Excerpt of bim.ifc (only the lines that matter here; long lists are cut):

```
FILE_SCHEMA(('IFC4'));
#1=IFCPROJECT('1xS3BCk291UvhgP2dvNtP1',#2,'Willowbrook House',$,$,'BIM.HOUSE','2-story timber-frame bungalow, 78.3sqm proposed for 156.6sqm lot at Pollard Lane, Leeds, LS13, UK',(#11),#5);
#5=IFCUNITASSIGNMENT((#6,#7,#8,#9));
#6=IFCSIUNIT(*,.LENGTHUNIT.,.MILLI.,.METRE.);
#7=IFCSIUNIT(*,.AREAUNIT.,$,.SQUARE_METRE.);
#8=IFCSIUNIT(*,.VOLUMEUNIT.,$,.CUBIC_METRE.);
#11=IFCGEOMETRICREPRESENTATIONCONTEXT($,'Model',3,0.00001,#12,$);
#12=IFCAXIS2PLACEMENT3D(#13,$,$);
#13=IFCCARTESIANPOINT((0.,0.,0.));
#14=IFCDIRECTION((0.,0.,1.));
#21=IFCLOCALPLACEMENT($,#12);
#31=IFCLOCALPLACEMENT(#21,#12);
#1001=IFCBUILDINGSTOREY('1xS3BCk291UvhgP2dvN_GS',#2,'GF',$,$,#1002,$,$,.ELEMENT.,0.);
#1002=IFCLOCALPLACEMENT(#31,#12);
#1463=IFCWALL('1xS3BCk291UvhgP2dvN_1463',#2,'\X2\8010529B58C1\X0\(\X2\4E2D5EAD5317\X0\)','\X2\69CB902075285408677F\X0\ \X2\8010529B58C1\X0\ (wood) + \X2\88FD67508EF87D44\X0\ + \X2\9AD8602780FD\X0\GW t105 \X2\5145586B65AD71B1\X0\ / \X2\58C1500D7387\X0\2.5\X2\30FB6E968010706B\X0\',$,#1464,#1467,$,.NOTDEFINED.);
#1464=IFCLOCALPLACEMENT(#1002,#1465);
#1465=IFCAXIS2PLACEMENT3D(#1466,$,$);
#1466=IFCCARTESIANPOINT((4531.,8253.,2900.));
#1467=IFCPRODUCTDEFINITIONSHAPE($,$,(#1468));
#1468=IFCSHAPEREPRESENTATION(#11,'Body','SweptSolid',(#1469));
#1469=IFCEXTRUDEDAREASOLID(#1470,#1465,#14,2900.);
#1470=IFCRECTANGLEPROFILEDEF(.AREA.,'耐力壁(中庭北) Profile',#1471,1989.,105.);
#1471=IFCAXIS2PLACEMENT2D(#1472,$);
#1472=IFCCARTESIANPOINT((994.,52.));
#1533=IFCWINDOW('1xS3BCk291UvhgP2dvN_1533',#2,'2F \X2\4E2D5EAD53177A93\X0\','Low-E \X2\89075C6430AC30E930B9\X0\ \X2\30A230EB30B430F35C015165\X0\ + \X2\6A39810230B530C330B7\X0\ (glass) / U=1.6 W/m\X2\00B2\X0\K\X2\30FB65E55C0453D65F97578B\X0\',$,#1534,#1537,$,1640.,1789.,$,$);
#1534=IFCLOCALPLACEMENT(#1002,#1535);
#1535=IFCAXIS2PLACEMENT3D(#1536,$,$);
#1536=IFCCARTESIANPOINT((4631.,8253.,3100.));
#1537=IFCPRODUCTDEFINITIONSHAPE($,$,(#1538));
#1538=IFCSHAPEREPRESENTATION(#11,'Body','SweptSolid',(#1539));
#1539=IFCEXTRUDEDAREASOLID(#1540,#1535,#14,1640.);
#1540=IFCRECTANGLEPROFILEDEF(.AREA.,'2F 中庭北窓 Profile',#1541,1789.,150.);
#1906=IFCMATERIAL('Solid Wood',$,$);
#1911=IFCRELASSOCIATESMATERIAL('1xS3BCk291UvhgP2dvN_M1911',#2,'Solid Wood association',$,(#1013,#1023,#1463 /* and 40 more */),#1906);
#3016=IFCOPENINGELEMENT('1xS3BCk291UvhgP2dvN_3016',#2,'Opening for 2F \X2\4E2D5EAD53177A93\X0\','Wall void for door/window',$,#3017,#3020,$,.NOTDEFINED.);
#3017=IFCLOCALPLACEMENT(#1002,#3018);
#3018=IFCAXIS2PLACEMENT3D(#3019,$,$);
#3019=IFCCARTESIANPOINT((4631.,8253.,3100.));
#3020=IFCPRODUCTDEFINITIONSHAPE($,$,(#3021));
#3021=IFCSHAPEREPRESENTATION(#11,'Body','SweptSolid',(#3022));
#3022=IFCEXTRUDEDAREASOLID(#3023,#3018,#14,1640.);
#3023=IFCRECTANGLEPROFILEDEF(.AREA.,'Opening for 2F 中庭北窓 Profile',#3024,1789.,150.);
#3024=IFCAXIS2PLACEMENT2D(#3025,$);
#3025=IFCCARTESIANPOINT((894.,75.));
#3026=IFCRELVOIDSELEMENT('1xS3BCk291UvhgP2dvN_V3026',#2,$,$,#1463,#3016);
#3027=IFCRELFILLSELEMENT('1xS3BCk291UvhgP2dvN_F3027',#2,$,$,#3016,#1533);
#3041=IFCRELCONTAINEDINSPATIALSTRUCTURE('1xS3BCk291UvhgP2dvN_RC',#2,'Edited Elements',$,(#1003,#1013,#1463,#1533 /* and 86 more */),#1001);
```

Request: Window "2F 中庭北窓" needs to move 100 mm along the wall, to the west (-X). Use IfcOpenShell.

```python
import ifcopenshell
import ifcopenshell.api.geometry
import ifcopenshell.util.placement
import ifcopenshell.util.unit

model = ifcopenshell.open("bim.ifc")
unit_scale = ifcopenshell.util.unit.calculate_unit_scale(model)

window = model.by_guid("1xS3BCk291UvhgP2dvN_1533")
opening = window.FillsVoids[0].RelatingOpeningElement
wall = opening.VoidsElements[0].RelatingBuildingElement

wall_matrix = ifcopenshell.util.placement.get_local_placement(wall.ObjectPlacement)
shift = wall_matrix[:3, 0] * -0.1 / unit_scale
before = ifcopenshell.util.placement.get_local_placement(window.ObjectPlacement)[:3, 3].copy()

# The window is not placed relative to its opening, so move both.
for product in (opening, window):
    matrix = ifcopenshell.util.placement.get_local_placement(product.ObjectPlacement)
    matrix[:3, 3] += shift
    ifcopenshell.api.geometry.edit_object_placement(model, product=product, matrix=matrix, is_si=False)

after = ifcopenshell.util.placement.get_local_placement(window.ObjectPlacement)[:3, 3]
print("window moved by", (after - before).round(3) + 0.0)

model.write("bim_v2.ifc")
```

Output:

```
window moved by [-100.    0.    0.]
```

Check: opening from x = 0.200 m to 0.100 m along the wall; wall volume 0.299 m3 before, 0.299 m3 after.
